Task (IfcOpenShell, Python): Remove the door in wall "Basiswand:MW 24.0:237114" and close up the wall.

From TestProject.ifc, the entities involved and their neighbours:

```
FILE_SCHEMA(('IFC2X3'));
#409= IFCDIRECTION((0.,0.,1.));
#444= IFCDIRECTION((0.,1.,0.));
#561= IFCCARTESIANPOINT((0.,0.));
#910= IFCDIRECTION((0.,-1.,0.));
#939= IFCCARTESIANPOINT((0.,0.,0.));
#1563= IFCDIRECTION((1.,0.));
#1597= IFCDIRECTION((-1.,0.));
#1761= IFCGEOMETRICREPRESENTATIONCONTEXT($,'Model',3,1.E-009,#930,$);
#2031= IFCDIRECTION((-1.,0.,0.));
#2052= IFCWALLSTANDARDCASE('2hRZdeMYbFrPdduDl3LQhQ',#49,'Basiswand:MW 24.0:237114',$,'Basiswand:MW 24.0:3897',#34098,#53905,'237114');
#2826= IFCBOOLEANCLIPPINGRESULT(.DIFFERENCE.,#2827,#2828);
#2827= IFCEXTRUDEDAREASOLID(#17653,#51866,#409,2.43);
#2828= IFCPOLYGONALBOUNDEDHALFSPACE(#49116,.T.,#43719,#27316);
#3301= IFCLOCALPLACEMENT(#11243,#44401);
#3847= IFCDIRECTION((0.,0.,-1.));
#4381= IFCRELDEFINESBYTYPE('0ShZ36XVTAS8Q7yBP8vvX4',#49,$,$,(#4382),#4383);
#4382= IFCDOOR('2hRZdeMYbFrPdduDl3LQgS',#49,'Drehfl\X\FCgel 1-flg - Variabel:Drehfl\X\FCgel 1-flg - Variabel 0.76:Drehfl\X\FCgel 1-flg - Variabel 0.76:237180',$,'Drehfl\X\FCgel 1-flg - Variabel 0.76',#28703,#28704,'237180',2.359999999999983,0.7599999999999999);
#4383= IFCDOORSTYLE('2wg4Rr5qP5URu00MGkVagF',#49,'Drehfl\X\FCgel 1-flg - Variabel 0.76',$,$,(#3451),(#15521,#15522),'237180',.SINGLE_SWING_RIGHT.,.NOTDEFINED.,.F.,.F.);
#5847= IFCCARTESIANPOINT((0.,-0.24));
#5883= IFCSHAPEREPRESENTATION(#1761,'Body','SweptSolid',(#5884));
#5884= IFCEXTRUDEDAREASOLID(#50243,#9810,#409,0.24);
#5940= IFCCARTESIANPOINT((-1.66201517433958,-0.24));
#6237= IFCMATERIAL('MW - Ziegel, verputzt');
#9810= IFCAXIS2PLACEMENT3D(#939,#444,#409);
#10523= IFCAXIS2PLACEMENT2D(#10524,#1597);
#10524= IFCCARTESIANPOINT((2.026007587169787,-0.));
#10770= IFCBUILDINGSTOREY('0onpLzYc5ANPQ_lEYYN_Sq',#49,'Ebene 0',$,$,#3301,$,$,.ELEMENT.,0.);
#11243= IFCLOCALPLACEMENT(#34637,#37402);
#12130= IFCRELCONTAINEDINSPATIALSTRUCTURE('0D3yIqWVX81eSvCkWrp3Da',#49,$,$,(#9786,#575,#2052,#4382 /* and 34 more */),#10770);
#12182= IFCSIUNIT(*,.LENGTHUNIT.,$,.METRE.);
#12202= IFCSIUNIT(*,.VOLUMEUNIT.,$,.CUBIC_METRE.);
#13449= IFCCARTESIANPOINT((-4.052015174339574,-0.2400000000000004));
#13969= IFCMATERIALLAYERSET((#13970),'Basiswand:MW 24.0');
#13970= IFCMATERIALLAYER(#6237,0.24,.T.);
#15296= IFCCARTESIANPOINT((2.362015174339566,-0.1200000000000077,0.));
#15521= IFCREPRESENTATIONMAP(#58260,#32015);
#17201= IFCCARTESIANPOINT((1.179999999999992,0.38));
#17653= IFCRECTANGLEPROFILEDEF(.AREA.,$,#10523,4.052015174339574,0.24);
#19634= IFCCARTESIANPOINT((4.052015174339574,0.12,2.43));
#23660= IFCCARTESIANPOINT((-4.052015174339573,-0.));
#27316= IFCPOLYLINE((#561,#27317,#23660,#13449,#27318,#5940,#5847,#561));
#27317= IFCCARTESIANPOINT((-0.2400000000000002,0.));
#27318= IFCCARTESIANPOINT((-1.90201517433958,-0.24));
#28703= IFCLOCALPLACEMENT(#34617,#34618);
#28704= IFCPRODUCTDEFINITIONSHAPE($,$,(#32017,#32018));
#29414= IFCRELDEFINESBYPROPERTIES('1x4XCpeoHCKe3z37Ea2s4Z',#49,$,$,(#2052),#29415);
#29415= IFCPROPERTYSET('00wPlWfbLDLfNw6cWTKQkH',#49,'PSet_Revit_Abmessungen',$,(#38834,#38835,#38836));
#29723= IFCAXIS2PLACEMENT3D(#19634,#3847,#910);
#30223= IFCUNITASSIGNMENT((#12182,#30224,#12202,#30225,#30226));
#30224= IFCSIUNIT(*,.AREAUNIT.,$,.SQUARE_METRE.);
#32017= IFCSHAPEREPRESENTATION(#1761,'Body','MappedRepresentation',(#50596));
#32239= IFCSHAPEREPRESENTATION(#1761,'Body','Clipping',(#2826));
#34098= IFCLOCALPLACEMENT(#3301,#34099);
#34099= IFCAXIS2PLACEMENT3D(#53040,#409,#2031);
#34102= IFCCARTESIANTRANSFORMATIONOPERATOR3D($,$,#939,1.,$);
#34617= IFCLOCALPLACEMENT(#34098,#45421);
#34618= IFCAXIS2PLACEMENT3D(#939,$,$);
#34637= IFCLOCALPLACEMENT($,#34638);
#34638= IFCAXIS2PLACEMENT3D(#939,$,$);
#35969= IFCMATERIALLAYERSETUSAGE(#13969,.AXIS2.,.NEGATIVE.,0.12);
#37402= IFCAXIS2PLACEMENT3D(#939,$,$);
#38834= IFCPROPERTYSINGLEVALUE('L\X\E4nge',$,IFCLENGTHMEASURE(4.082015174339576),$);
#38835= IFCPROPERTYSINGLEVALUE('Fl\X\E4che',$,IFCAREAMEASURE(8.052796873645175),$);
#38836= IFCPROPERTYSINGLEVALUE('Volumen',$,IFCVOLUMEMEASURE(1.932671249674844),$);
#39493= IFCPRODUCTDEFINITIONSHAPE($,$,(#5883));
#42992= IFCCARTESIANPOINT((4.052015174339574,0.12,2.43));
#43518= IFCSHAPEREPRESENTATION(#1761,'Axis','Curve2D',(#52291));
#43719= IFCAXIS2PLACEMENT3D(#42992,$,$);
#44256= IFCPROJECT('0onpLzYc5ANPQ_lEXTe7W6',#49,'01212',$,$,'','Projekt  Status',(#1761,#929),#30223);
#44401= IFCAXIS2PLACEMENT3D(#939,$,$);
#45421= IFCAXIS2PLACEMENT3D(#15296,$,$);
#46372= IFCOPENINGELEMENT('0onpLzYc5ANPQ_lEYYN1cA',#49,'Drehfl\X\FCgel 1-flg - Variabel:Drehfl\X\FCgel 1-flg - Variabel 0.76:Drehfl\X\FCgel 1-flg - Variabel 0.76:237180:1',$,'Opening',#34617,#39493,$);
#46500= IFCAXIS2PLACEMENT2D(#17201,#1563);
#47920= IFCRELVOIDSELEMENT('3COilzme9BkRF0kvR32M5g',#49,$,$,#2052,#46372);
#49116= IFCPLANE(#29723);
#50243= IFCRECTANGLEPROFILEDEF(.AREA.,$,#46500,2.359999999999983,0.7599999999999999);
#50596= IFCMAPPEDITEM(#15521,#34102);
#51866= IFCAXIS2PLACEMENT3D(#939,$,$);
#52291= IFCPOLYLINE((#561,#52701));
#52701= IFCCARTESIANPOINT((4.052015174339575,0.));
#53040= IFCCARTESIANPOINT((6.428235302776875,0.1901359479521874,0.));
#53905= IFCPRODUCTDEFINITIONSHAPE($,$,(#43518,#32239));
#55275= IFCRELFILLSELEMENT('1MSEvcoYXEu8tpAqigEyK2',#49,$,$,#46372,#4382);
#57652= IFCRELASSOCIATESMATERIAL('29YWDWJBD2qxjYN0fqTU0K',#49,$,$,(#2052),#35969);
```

```python
import ifcopenshell
import ifcopenshell.api.feature
import ifcopenshell.api.pset
import ifcopenshell.api.root
import ifcopenshell.geom
import ifcopenshell.util.element
import ifcopenshell.util.shape
import ifcopenshell.util.unit

model = ifcopenshell.open("TestProject.ifc")
area_scale = ifcopenshell.util.unit.calculate_unit_scale(model, "AREAUNIT")
volume_scale = ifcopenshell.util.unit.calculate_unit_scale(model, "VOLUMEUNIT")
settings = ifcopenshell.geom.settings()


def volume(element):
    """Net volume in cubic metres, openings subtracted."""
    shape = ifcopenshell.geom.create_shape(settings, element)
    return ifcopenshell.util.shape.get_volume(shape.geometry)


door = model.by_guid("2hRZdeMYbFrPdduDl3LQgS")
opening = door.FillsVoids[0].RelatingOpeningElement
wall = opening.VoidsElements[0].RelatingBuildingElement
before = volume(wall)

ifcopenshell.api.root.remove_product(model, product=door)
ifcopenshell.api.feature.remove_feature(model, feature=opening)

after = volume(wall)
thickness = 0.24  # wall thickness in metres

# Update the wall's stored quantities.
pset = model.by_id(ifcopenshell.util.element.get_pset(wall, "PSet_Revit_Abmessungen", should_inherit=False)["id"])
ifcopenshell.api.pset.edit_pset(model, pset=pset, properties={
    "Fläche": model.create_entity("IfcAreaMeasure", after / thickness / area_scale),
    "Volumen": model.create_entity("IfcVolumeMeasure", after / volume_scale),
})

print(f"wall volume {before:.3f} -> {after:.3f} m3")

model.write("TestProject_rev.ifc")
```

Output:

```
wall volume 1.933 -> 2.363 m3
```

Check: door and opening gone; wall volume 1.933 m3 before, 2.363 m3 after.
